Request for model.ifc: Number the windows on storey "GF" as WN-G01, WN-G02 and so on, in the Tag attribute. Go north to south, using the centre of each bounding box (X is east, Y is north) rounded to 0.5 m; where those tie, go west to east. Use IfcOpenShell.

First a look at what the model holds.

```python
import ifcopenshell
import ifcopenshell.util.element
import ifcopenshell.util.placement

model = ifcopenshell.open("model.ifc")
print(model.schema)
storey = next(s for s in model.by_type("IfcBuildingStorey") if s.Name == "GF")
windows = [e for e in ifcopenshell.util.element.get_decomposition(storey) if e.is_a("IfcWindow")]
for e in sorted(windows, key=lambda e: e.id()):
    origin = ifcopenshell.util.placement.get_local_placement(e.ObjectPlacement)[:3, 3]
    print(e.id(), e.Tag, e.Name, origin.round(2) + 0.0, sep=" | ")
```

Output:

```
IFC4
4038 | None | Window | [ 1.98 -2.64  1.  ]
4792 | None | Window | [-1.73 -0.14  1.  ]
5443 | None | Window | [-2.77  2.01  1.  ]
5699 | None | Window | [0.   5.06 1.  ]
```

```python
import ifcopenshell
import ifcopenshell.geom
import ifcopenshell.util.element
import ifcopenshell.util.shape

model = ifcopenshell.open("model.ifc")
settings = ifcopenshell.geom.settings()
settings.set("use-world-coords", True)


def centre(element):
    shape = ifcopenshell.geom.create_shape(settings, element)
    return ifcopenshell.util.shape.get_bbox_centroid(shape.geometry)


storey = next(s for s in model.by_type("IfcBuildingStorey") if s.Name == "GF")
windows = [e for e in ifcopenshell.util.element.get_decomposition(storey) if e.is_a("IfcWindow")]

# Insertion points can sit at a corner or the storey origin, so sort by the geometry (in metres).
centres = {e: centre(e) for e in windows}
windows.sort(key=lambda e: (-round(centres[e][1] / 0.5), centres[e][0]))

for i, e in enumerate(windows, start=1):
    number = f"WN-G{i:02d}"
    e.Tag = number
    print(e.id(), number)

model.write("model_rev.ifc")
```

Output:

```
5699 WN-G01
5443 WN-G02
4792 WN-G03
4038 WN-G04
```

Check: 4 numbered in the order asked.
